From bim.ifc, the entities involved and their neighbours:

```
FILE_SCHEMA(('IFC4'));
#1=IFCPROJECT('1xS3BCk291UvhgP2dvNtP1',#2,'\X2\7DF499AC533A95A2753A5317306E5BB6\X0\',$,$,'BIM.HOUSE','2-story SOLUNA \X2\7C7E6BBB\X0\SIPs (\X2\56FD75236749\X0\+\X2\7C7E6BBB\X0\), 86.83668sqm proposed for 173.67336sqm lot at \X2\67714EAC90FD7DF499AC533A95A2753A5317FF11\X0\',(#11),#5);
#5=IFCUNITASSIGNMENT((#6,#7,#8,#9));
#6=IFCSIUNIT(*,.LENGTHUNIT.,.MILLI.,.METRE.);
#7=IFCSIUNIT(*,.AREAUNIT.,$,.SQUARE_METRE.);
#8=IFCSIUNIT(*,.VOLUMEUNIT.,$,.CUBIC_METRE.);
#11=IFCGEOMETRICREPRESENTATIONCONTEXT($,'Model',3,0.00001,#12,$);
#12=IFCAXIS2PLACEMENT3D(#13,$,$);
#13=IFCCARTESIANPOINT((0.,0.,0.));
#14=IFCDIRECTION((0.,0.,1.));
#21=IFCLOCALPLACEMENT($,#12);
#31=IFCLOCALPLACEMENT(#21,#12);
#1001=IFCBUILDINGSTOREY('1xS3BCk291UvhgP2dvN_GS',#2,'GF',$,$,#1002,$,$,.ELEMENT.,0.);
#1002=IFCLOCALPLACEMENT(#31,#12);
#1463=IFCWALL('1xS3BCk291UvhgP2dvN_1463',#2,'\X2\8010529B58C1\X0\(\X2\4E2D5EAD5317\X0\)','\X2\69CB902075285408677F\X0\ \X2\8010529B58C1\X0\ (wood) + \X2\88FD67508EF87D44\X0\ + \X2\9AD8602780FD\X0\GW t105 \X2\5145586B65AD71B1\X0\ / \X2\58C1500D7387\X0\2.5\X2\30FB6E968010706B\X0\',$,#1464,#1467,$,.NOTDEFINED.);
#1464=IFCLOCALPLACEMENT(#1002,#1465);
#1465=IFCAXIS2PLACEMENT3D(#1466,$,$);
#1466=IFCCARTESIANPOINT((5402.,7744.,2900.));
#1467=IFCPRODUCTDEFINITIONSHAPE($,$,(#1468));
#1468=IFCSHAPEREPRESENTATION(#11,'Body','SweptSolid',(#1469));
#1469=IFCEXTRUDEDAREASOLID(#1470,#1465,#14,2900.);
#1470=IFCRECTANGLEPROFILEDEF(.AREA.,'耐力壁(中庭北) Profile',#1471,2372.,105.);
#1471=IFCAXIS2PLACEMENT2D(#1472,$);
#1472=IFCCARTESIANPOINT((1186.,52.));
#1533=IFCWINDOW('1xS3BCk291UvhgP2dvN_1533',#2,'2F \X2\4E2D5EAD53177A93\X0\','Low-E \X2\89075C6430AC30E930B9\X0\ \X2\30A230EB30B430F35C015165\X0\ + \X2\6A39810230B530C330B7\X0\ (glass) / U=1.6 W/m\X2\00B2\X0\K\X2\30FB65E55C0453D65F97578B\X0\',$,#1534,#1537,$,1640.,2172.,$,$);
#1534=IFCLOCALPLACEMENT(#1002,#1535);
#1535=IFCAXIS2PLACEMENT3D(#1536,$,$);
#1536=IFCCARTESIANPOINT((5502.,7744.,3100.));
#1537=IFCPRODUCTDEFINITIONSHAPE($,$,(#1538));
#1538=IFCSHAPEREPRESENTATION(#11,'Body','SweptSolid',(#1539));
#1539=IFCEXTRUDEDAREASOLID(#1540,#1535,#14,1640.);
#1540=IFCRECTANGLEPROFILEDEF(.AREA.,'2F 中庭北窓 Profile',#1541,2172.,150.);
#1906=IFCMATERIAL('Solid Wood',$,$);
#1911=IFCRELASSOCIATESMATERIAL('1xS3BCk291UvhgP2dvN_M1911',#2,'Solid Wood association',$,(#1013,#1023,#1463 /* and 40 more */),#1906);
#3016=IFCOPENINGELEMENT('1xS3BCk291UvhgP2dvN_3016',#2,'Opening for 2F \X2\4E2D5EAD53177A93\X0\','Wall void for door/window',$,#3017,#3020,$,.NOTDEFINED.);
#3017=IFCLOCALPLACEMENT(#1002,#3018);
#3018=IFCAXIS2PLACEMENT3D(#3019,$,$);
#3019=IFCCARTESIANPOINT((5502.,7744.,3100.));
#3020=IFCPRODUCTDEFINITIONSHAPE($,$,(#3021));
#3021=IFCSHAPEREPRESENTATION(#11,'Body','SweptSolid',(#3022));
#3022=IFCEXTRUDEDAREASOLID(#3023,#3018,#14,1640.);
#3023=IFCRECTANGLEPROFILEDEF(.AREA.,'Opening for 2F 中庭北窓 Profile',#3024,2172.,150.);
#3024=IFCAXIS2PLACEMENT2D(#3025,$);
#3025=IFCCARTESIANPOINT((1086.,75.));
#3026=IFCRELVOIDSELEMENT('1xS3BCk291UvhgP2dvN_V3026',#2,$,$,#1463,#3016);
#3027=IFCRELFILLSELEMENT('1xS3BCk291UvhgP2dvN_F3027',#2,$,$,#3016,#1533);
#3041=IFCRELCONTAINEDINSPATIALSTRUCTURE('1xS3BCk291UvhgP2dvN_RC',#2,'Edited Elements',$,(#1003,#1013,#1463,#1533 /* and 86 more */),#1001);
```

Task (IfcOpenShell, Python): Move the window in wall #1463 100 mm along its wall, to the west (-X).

```python
import ifcopenshell
import ifcopenshell.api.geometry
import ifcopenshell.util.placement
import ifcopenshell.util.unit

model = ifcopenshell.open("bim.ifc")
unit_scale = ifcopenshell.util.unit.calculate_unit_scale(model)

window = model.by_guid("1xS3BCk291UvhgP2dvN_1533")
opening = window.FillsVoids[0].RelatingOpeningElement
wall = opening.VoidsElements[0].RelatingBuildingElement

wall_matrix = ifcopenshell.util.placement.get_local_placement(wall.ObjectPlacement)
shift = wall_matrix[:3, 0] * -0.1 / unit_scale
before = ifcopenshell.util.placement.get_local_placement(window.ObjectPlacement)[:3, 3].copy()

# The window is not placed relative to its opening, so move both.
for product in (opening, window):
    matrix = ifcopenshell.util.placement.get_local_placement(product.ObjectPlacement)
    matrix[:3, 3] += shift
    ifcopenshell.api.geometry.edit_object_placement(model, product=product, matrix=matrix, is_si=False)

after = ifcopenshell.util.placement.get_local_placement(window.ObjectPlacement)[:3, 3]
print("window moved by", (after - before).round(3) + 0.0)

model.write("bim_updated.ifc")
```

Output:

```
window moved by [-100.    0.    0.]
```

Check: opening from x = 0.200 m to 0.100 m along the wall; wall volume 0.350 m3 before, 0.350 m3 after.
